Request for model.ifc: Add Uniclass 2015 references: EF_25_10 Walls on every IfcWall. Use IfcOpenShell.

First a look at what the model holds.

```python
import ifcopenshell

model = ifcopenshell.open("model.ifc")
print(model.schema)
print("classifications:", [c.Name for c in model.by_type("IfcClassification")])
for ifc_class in ("IfcDoor", "IfcRoof", "IfcStair", "IfcWall", "IfcWindow"):
    print(ifc_class, len(model.by_type(ifc_class)))
```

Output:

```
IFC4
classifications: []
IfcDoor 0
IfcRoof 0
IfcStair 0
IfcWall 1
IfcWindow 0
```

```python
import ifcopenshell
import ifcopenshell.api.classification

model = ifcopenshell.open("model.ifc")

system = ifcopenshell.api.classification.add_classification(model, classification="Uniclass 2015")

codes = {
    "IfcWall": ("EF_25_10", "Walls"),
}
for ifc_class, (code, name) in codes.items():
    products = model.by_type(ifc_class)
    ifcopenshell.api.classification.add_reference(
        model, products=products, classification=system, identification=code, name=name
    )
    print(code, len(products))

model.write("model-out.ifc")
```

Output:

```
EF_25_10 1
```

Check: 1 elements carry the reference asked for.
